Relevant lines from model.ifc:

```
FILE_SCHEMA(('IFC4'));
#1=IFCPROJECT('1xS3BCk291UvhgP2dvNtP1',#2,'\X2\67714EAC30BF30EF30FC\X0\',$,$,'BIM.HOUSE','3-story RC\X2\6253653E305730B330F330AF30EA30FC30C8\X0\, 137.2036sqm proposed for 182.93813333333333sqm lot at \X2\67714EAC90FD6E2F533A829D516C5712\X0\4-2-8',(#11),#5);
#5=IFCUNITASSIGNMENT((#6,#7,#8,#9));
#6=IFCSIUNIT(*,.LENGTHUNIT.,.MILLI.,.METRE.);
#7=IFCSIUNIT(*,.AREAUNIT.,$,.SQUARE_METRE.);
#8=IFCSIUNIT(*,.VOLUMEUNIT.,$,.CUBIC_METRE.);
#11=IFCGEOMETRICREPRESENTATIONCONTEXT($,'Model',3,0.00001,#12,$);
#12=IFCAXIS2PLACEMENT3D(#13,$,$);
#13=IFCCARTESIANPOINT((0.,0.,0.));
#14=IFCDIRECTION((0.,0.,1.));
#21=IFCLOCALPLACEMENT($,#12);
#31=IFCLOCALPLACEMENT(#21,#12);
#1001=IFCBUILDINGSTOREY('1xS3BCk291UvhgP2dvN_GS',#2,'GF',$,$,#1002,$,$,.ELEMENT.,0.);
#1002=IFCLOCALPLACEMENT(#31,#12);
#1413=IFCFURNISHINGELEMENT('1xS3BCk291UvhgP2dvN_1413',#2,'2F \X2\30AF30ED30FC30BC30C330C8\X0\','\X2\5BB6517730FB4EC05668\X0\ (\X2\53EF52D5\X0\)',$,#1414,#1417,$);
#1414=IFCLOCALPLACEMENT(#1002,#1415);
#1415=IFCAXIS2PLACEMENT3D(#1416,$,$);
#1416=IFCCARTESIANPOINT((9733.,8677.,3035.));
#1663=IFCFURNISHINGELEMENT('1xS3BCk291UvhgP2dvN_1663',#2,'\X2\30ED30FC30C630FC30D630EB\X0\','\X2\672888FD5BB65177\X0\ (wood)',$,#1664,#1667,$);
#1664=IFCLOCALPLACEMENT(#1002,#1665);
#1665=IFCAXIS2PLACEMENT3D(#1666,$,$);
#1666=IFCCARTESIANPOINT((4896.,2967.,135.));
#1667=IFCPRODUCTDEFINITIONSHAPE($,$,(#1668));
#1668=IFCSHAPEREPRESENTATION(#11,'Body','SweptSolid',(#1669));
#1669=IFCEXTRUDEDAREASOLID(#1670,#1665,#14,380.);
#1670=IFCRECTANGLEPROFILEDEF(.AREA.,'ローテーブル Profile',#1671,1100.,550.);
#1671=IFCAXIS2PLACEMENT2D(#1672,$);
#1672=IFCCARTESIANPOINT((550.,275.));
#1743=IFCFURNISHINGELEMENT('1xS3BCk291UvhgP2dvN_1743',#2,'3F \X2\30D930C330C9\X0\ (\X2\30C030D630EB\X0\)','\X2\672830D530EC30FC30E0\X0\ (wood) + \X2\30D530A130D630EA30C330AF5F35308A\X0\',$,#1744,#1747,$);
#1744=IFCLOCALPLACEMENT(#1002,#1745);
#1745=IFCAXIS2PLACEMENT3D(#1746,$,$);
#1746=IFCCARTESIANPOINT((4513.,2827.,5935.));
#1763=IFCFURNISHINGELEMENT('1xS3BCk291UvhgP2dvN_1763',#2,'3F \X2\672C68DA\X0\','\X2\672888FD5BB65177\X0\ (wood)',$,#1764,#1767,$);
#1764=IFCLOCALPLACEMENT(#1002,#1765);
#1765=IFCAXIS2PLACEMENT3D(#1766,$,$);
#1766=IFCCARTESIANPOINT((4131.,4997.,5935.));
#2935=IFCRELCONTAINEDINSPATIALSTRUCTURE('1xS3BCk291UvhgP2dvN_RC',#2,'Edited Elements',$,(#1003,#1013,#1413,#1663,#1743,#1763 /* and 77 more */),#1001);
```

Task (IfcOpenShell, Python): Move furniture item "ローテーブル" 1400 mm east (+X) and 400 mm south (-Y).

```python
import ifcopenshell
import ifcopenshell.api.geometry
import ifcopenshell.util.placement
import ifcopenshell.util.unit

model = ifcopenshell.open("model.ifc")
unit_scale = ifcopenshell.util.unit.calculate_unit_scale(model)

item = model.by_id(1663)
matrix = ifcopenshell.util.placement.get_local_placement(item.ObjectPlacement)
matrix[0, 3] += 1.4 / unit_scale
matrix[1, 3] -= 0.4 / unit_scale
ifcopenshell.api.geometry.edit_object_placement(model, product=item, matrix=matrix, is_si=False)

print(ifcopenshell.util.placement.get_local_placement(item.ObjectPlacement).round(3) + 0.0)

model.write("model-out.ifc")
```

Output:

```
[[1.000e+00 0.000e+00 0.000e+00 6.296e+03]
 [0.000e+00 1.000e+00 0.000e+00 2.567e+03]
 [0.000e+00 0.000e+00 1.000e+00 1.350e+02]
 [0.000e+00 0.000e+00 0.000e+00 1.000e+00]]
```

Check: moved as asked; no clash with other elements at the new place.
